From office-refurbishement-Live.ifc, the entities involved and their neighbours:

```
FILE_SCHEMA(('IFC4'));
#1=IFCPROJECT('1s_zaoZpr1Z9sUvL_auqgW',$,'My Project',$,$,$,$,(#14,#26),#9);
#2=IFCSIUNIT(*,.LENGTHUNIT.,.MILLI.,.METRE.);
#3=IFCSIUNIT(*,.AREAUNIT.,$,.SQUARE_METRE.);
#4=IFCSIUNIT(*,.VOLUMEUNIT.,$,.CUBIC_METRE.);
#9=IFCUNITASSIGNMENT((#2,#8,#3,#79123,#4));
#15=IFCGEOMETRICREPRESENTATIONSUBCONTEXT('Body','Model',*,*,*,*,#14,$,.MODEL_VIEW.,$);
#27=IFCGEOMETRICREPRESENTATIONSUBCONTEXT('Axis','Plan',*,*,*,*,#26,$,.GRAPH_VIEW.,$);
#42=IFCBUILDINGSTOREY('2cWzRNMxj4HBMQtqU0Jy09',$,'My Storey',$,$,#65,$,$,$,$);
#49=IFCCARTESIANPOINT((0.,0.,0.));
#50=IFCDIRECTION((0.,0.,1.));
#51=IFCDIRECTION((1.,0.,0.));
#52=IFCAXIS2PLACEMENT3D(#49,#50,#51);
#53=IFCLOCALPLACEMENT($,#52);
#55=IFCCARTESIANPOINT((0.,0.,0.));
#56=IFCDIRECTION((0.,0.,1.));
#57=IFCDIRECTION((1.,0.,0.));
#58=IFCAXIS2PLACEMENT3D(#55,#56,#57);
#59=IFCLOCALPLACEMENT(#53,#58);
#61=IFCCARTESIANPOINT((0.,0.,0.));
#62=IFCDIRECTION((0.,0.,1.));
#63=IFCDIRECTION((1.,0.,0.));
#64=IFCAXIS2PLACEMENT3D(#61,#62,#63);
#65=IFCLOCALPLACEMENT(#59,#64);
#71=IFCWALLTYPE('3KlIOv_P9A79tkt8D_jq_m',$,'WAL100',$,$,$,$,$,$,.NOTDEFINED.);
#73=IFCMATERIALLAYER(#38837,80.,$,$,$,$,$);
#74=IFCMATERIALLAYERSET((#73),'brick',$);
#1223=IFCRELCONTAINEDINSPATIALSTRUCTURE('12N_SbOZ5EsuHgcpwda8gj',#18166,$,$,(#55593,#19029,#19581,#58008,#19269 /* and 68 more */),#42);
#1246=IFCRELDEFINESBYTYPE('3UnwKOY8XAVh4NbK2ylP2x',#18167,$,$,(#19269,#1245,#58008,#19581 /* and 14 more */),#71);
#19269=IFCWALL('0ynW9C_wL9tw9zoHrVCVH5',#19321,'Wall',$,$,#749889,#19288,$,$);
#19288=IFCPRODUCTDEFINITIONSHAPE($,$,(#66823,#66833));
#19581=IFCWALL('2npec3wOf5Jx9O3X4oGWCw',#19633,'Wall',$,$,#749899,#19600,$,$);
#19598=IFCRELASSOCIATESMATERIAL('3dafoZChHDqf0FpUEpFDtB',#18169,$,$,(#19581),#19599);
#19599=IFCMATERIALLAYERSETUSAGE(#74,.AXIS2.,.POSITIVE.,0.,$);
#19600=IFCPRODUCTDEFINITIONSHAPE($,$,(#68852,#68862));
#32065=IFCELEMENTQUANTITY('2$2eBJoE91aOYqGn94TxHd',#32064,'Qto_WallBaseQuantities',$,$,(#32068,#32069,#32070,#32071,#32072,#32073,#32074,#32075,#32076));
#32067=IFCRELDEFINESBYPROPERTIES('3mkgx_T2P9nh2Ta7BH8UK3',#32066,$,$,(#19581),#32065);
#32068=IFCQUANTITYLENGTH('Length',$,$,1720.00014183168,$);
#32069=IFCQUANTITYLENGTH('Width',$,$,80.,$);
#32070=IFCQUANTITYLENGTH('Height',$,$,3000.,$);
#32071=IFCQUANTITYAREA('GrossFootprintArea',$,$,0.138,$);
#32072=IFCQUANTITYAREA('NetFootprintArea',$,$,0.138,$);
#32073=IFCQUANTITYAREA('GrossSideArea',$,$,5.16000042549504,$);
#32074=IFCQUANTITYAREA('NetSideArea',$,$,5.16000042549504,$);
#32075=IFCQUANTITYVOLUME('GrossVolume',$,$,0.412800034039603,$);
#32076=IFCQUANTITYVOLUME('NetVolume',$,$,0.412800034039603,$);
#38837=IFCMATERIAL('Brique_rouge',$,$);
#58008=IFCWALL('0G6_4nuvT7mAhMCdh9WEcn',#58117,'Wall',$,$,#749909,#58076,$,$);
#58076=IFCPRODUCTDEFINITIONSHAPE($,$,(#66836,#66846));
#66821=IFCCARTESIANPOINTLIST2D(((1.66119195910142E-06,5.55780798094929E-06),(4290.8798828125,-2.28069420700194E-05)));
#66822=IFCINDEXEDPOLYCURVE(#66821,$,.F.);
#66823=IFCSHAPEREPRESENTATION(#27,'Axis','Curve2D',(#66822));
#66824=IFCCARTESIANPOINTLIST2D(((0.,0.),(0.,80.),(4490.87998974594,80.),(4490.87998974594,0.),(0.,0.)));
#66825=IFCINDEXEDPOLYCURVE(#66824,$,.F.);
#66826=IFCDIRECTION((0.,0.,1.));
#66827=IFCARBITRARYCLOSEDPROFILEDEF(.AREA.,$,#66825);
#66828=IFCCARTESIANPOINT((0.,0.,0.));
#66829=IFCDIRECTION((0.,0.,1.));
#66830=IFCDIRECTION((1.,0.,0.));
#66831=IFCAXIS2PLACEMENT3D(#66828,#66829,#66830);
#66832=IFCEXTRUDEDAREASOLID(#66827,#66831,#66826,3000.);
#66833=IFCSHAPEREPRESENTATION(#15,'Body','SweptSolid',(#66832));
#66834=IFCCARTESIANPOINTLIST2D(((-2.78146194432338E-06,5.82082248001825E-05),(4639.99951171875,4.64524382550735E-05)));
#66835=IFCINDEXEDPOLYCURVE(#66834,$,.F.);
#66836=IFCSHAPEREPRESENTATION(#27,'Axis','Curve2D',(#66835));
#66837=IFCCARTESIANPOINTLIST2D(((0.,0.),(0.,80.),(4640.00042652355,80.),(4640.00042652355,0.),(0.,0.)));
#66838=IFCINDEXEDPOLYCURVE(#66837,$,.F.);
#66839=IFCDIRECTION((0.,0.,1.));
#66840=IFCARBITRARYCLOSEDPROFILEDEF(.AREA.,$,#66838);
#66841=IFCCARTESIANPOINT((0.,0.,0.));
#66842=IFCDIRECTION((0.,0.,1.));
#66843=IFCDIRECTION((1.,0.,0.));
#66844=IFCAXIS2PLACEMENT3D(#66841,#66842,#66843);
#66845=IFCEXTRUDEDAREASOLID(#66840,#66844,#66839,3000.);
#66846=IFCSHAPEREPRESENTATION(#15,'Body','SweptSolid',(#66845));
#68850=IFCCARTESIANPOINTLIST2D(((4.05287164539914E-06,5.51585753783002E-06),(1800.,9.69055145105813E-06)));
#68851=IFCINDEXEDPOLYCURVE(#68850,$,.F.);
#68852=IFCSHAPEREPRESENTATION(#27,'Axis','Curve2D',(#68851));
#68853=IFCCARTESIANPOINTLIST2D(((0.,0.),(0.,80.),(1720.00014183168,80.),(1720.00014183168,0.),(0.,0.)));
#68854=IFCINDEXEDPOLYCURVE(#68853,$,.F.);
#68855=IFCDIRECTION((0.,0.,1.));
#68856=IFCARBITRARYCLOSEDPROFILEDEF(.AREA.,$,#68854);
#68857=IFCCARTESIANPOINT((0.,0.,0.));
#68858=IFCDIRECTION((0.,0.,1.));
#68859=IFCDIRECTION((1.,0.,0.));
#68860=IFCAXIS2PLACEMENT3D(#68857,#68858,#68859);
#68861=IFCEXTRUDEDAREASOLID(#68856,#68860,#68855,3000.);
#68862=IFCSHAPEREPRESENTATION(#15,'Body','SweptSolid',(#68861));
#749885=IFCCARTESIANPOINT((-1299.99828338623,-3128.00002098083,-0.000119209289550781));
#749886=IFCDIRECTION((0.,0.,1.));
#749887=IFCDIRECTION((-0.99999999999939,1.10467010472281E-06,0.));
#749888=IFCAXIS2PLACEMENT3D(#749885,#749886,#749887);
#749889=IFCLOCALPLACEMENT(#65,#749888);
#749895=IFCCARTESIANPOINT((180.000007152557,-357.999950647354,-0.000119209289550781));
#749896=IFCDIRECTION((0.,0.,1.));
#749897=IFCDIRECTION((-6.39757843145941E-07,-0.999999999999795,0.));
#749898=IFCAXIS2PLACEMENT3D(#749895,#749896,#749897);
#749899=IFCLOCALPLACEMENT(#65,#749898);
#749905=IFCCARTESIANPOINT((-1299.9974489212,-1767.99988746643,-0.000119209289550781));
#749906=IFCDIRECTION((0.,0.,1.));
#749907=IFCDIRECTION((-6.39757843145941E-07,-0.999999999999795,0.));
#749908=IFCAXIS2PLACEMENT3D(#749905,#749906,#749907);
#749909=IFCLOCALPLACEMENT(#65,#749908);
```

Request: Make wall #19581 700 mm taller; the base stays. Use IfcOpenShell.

```python
import ifcopenshell
import ifcopenshell.api.pset
import ifcopenshell.geom
import ifcopenshell.util.element
import ifcopenshell.util.representation
import ifcopenshell.util.shape
import ifcopenshell.util.unit

model = ifcopenshell.open("office-refurbishement-Live.ifc")
unit_scale = ifcopenshell.util.unit.calculate_unit_scale(model)
area_scale = ifcopenshell.util.unit.calculate_unit_scale(model, "AREAUNIT")
volume_scale = ifcopenshell.util.unit.calculate_unit_scale(model, "VOLUMEUNIT")
settings = ifcopenshell.geom.settings()


def volume(element):
    """Net volume in cubic metres, openings subtracted."""
    shape = ifcopenshell.geom.create_shape(settings, element)
    return ifcopenshell.util.shape.get_volume(shape.geometry)


wall = model.by_guid("2npec3wOf5Jx9O3X4oGWCw")
before = volume(wall)

body = ifcopenshell.util.representation.get_representation(wall, "Model", "Body")
solid = body.Items[0]
old_height = solid.Depth
solid.Depth += 700.0
after = volume(wall)
thickness = 0.08  # wall thickness in metres

# Update the stored height, areas and volumes.
qto = model.by_id(ifcopenshell.util.element.get_pset(wall, "Qto_WallBaseQuantities", should_inherit=False)["id"])
ifcopenshell.api.pset.edit_qto(model, qto=qto, properties={
    "Height": solid.Depth,
    "GrossSideArea": ifcopenshell.util.element.get_pset(wall, "Qto_WallBaseQuantities", "GrossSideArea") * solid.Depth / old_height,
    "NetSideArea": after / thickness / area_scale,
    "GrossVolume": ifcopenshell.util.element.get_pset(wall, "Qto_WallBaseQuantities", "GrossVolume") * solid.Depth / old_height,
    "NetVolume": after / volume_scale,
})

print(f"height {old_height:g} -> {solid.Depth:g}, volume {before:.3f} -> {after:.3f} m3")

model.write("office-refurbishement-Live-out.ifc")
```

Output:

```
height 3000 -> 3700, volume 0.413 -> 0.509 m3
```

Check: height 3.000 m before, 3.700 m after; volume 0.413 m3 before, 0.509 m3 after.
